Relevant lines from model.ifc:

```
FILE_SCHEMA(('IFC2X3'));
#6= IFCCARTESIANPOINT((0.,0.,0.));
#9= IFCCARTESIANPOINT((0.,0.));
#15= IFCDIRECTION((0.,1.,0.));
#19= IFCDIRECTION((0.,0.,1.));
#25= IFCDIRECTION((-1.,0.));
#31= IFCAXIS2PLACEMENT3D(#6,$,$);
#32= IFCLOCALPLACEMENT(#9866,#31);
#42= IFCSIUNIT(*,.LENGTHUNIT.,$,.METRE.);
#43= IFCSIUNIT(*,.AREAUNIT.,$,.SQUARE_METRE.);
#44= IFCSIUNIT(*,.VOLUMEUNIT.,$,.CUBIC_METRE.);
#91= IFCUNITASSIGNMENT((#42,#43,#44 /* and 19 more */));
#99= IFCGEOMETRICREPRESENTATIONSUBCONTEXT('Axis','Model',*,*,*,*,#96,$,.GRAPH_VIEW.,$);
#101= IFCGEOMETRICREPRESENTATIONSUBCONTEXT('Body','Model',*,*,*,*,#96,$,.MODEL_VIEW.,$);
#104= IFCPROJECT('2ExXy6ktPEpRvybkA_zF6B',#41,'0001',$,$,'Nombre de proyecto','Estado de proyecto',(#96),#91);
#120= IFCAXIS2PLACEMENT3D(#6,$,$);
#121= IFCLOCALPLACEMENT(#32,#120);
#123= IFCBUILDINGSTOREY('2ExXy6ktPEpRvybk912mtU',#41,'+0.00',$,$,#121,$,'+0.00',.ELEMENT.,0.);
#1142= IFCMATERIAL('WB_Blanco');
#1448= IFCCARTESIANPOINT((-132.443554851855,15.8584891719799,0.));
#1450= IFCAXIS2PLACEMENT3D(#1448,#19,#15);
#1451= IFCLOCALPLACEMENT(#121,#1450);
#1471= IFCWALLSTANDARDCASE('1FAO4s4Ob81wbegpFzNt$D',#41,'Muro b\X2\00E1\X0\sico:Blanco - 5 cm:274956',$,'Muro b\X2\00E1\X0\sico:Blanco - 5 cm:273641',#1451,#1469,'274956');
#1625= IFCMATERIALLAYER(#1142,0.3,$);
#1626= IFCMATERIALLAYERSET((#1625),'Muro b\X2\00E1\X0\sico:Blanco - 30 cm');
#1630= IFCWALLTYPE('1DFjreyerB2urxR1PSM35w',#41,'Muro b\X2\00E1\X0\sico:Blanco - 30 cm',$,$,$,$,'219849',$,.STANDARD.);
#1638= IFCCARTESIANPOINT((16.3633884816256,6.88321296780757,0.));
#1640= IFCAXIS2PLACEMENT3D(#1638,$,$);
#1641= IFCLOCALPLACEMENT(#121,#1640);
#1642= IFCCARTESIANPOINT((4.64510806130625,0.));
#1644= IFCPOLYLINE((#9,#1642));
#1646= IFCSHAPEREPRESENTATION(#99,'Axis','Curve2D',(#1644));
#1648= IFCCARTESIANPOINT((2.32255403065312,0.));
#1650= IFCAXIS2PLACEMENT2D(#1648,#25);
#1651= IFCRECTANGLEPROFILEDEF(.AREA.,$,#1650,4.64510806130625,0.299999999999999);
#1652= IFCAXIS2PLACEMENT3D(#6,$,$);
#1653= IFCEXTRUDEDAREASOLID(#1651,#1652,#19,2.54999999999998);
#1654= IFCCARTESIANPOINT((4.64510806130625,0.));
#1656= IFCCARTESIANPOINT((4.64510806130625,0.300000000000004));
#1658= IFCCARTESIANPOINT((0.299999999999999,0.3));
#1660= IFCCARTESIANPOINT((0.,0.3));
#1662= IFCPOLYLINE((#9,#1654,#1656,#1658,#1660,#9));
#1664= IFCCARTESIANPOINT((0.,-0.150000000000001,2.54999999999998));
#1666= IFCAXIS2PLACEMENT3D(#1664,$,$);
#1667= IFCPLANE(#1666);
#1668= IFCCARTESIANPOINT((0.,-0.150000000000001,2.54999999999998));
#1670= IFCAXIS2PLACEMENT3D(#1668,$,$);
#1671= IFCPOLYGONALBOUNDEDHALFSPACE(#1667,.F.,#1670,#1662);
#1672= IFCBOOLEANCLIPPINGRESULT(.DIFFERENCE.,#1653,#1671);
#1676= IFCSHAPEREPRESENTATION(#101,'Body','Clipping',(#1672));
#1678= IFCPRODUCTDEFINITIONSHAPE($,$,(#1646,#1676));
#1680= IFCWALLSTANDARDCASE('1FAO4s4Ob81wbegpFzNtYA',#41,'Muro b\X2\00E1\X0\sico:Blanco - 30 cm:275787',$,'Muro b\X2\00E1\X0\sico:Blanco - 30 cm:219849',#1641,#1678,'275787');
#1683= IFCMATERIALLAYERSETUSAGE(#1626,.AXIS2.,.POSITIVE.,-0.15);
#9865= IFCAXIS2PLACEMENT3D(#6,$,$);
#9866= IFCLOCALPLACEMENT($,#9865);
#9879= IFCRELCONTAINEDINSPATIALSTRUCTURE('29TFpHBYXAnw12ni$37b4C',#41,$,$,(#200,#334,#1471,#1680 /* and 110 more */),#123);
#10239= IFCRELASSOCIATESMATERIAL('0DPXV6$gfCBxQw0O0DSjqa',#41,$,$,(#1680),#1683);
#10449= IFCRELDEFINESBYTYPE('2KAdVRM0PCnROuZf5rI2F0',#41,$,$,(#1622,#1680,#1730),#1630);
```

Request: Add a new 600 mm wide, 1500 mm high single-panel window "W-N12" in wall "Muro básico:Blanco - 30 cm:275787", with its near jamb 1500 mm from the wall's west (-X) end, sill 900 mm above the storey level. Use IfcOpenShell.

```python
import numpy as np
import ifcopenshell
import ifcopenshell.api.feature
import ifcopenshell.api.geometry
import ifcopenshell.api.root
import ifcopenshell.api.spatial
import ifcopenshell.api.type
import ifcopenshell.geom
import ifcopenshell.util.element
import ifcopenshell.util.placement
import ifcopenshell.util.representation
import ifcopenshell.util.shape
import ifcopenshell.util.unit

model = ifcopenshell.open("model.ifc")
unit_scale = ifcopenshell.util.unit.calculate_unit_scale(model)
settings = ifcopenshell.geom.settings()


def volume(element):
    """Net volume in cubic metres, openings subtracted."""
    shape = ifcopenshell.geom.create_shape(settings, element)
    return ifcopenshell.util.shape.get_volume(shape.geometry)


wall = model.by_guid("1FAO4s4Ob81wbegpFzNtYA")
storey = ifcopenshell.util.element.get_container(wall, ifc_class="IfcBuildingStorey")
context = ifcopenshell.util.representation.get_context(model, "Model", "Body", "MODEL_VIEW")
before = volume(wall)

width, height, from_end, sill = 0.6, 1.5, 1.5, 0.9  # metres

# The wall runs along its own X axis, and the end named is its -X end.
wall_shape = ifcopenshell.geom.create_shape(settings, wall)
x, y, z = ifcopenshell.util.shape.get_vertices(wall_shape.geometry).T
start = x.min() + from_end
face, thickness = float(y.min()), float(y.max() - y.min())
wall_matrix = ifcopenshell.util.placement.get_local_placement(wall.ObjectPlacement)
level = ifcopenshell.util.placement.get_local_placement(storey.ObjectPlacement)[2, 3]


def in_wall(x, y):
    """Placement at x, y metres in the wall's axes, at sill height."""
    matrix = wall_matrix.copy()
    matrix[:, 3] = wall_matrix @ np.array([x / unit_scale, y / unit_scale, 0.0, 1.0])
    matrix[2, 3] = level + sill / unit_scale
    return matrix


# Opening: a box that overshoots both wall faces by 50 mm.
opening = ifcopenshell.api.root.create_entity(model, ifc_class="IfcOpeningElement")
box = ifcopenshell.api.geometry.add_wall_representation(
    model, context=context, length=width, height=height, thickness=thickness + 0.1
)
ifcopenshell.api.geometry.assign_representation(model, product=opening, representation=box)
ifcopenshell.api.geometry.edit_object_placement(model, product=opening, matrix=in_wall(start, face - 0.05), is_si=False)
ifcopenshell.api.feature.add_feature(model, feature=opening, element=wall)

window = ifcopenshell.api.root.create_entity(model, ifc_class="IfcWindow", name="W-N12")
window.OverallWidth, window.OverallHeight = width / unit_scale, height / unit_scale
body = ifcopenshell.api.geometry.add_window_representation(
    model,
    context=context,
    overall_width=window.OverallWidth,
    overall_height=window.OverallHeight,
    partition_type="SINGLE_PANEL",
)
ifcopenshell.api.geometry.assign_representation(model, product=window, representation=body)
ifcopenshell.api.spatial.assign_container(model, products=[window], relating_structure=storey)
fills = ifcopenshell.api.feature.add_filling(model, opening=opening, element=window)
fills.OwnerHistory = window.OwnerHistory  # required in IFC2X3

# IFC2X3 keeps the operation on the window style.
style = ifcopenshell.api.root.create_entity(model, ifc_class="IfcWindowStyle", name="W-N12")
style.OperationType, style.ConstructionType = "SINGLE_PANEL", "NOTDEFINED"
style.ParameterTakesPrecedence = style.Sizeable = False
ifcopenshell.api.type.assign_type(model, related_objects=[window], relating_type=style)

# Centre the window in the wall's thickness.
ifcopenshell.api.geometry.edit_object_placement(model, product=window, matrix=in_wall(start, face), is_si=False)
window_shape = ifcopenshell.geom.create_shape(settings, window)
depth = ifcopenshell.util.shape.get_vertices(window_shape.geometry)[:, 1]
offset = face + thickness / 2 - (depth.min() + depth.max()) / 2
ifcopenshell.api.geometry.edit_object_placement(model, product=window, matrix=in_wall(start, offset), is_si=False)

after = volume(wall)

print(f"wall volume {before:.3f} -> {after:.3f} m3")

model.write("model_rev.ifc")
```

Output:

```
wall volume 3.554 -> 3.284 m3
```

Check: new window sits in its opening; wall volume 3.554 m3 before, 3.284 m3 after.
